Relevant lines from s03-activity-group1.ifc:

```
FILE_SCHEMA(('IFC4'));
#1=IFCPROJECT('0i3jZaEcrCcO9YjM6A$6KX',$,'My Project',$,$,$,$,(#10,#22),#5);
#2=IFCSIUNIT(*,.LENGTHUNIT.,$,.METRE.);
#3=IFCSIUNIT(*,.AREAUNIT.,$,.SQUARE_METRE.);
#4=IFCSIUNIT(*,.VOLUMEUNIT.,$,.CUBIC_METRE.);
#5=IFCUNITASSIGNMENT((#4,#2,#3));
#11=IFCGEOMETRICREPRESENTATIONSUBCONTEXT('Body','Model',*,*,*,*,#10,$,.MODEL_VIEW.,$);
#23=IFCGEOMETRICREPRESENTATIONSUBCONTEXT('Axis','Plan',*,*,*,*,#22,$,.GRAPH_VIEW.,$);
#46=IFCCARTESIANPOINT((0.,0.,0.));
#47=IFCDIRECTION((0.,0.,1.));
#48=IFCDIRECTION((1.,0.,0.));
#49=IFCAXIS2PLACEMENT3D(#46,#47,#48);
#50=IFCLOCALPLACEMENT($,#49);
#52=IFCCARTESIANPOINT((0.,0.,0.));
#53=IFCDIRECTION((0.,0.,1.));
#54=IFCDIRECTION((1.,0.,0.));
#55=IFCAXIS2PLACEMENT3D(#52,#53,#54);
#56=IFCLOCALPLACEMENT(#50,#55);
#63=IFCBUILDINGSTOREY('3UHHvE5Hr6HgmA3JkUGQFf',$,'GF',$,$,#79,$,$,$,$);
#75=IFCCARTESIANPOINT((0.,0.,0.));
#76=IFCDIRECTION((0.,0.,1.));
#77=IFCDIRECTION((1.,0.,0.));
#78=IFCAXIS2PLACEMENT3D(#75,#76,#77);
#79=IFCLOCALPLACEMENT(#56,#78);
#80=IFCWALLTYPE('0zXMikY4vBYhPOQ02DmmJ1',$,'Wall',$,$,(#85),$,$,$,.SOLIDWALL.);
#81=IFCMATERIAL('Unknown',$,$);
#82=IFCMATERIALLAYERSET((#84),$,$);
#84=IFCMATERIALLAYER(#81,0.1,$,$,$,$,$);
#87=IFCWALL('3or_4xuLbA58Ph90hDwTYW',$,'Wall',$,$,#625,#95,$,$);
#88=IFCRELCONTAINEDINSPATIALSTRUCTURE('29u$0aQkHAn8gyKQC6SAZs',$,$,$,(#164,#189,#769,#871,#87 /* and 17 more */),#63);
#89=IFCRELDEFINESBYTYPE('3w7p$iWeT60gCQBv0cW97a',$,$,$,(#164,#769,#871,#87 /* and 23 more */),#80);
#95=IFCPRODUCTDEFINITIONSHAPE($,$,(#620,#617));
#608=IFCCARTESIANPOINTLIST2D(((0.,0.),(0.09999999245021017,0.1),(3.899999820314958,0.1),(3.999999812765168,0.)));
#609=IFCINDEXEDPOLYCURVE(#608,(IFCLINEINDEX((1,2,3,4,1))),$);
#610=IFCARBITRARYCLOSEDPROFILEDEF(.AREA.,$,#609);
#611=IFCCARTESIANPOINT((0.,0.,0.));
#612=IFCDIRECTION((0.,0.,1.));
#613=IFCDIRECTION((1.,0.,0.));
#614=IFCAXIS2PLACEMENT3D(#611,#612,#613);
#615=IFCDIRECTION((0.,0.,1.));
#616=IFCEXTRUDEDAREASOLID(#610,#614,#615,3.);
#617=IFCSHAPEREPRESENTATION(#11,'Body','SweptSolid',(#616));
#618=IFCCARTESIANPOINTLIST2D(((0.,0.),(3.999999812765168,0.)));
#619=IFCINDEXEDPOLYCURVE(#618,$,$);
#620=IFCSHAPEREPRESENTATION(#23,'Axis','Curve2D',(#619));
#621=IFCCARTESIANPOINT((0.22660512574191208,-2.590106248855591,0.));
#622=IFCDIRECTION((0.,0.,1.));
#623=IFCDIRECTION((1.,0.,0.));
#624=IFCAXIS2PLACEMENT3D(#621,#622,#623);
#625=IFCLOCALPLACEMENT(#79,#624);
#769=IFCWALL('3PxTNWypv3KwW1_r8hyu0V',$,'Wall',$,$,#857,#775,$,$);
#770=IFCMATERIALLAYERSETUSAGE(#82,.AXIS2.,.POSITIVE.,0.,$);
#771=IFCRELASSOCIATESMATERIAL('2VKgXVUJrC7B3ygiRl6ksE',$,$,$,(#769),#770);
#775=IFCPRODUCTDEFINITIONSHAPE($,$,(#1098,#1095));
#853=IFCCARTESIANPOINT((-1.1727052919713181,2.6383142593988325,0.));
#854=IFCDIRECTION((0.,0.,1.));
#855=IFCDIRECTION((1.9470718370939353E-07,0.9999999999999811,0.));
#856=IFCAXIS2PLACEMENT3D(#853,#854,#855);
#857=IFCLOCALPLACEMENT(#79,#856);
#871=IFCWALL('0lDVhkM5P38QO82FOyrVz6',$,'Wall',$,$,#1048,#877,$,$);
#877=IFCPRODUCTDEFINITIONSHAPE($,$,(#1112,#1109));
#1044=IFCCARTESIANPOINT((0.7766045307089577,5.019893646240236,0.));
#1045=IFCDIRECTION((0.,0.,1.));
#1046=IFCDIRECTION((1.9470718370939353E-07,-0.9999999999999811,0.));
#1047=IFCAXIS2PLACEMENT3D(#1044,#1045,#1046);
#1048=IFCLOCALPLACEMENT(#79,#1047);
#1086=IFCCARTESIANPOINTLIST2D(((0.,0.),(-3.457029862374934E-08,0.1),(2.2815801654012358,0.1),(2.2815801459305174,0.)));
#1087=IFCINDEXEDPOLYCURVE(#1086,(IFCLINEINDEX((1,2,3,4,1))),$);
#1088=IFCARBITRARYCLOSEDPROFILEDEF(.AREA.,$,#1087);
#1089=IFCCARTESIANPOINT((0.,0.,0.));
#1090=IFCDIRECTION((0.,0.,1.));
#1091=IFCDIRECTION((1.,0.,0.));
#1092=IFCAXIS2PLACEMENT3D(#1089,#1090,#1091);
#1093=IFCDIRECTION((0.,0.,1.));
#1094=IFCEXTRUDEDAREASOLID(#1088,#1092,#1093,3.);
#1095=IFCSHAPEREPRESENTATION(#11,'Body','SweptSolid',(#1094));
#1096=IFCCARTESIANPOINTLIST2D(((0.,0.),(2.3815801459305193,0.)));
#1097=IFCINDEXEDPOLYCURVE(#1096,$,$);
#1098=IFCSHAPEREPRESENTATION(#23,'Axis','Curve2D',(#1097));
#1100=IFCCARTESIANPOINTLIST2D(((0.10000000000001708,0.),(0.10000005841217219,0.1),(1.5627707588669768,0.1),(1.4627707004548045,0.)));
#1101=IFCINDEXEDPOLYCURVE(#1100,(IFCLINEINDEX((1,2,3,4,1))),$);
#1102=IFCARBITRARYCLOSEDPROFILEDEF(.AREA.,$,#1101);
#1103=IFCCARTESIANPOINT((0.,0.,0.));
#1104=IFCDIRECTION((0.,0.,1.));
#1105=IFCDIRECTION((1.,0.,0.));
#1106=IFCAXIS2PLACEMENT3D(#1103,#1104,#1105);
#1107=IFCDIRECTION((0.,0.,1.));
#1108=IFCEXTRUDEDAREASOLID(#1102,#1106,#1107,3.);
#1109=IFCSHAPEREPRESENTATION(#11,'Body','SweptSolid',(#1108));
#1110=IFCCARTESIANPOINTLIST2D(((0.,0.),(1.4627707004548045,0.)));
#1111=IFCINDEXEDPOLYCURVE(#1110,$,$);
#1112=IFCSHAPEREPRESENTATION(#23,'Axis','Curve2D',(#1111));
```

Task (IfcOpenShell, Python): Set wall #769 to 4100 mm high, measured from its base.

```python
import ifcopenshell
import ifcopenshell.geom
import ifcopenshell.util.representation
import ifcopenshell.util.shape
import ifcopenshell.util.unit

model = ifcopenshell.open("s03-activity-group1.ifc")
unit_scale = ifcopenshell.util.unit.calculate_unit_scale(model)
settings = ifcopenshell.geom.settings()


def volume(element):
    """Net volume in cubic metres, openings subtracted."""
    shape = ifcopenshell.geom.create_shape(settings, element)
    return ifcopenshell.util.shape.get_volume(shape.geometry)


wall = model.by_guid("3PxTNWypv3KwW1_r8hyu0V")
before = volume(wall)

body = ifcopenshell.util.representation.get_representation(wall, "Model", "Body")
solid = body.Items[0]
old_height = solid.Depth
solid.Depth = 4.1 / unit_scale
after = volume(wall)

print(f"height {old_height:g} -> {solid.Depth:g}, volume {before:.3f} -> {after:.3f} m3")

model.write("s03-activity-group1-out.ifc")
```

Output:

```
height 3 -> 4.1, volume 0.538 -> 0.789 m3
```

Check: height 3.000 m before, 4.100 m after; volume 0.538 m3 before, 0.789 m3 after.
